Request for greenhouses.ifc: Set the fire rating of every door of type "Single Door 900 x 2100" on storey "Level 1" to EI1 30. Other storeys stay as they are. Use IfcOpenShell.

First a look at what the model holds.

```python
import ifcopenshell
import ifcopenshell.util.element

model = ifcopenshell.open("greenhouses.ifc")
print(model.schema)
storey = next(s for s in model.by_type("IfcBuildingStorey") if s.Name == "Level 1")
doors = [e for e in ifcopenshell.util.element.get_decomposition(storey) if e.is_a("IfcDoor")]
seen = {}
for e in doors:
    element_type = ifcopenshell.util.element.get_type(e)
    key = (element_type.Name if element_type != e and element_type else None, ifcopenshell.util.element.get_pset(e, "Pset_DoorCommon", "FireRating"))
    seen[key] = seen.get(key, 0) + 1
for (name, value), count in sorted(seen.items(), key=str):
    print(count, "x", name, "|", value)
```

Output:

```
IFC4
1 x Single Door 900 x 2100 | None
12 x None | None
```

```python
import ifcopenshell
import ifcopenshell.api.pset
import ifcopenshell.util.element

model = ifcopenshell.open("greenhouses.ifc")

storey = next(s for s in model.by_type("IfcBuildingStorey") if s.Name == "Level 1")
doors = [e for e in ifcopenshell.util.element.get_decomposition(storey) if e.is_a("IfcDoor")]

count = 0
for e in doors:
    element_type = ifcopenshell.util.element.get_type(e)
    if element_type in (None, e) or element_type.Name != "Single Door 900 x 2100":
        continue
    # add_pset returns the element's existing set when there is one.
    pset = ifcopenshell.api.pset.add_pset(model, product=e, name="Pset_DoorCommon")
    ifcopenshell.api.pset.edit_pset(model, pset=pset, properties={"FireRating": "EI1 30"})
    count += 1

print(count, "doors updated")

model.write("greenhouses_rev.ifc")
```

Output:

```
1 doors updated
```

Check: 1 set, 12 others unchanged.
